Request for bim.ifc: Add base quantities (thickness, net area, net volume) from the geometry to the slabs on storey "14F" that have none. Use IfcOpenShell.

First a look at what the model holds.

```python
import ifcopenshell
import ifcopenshell.util.element
import ifcopenshell.util.unit

model = ifcopenshell.open("bim.ifc")
print(model.schema)
for unit_type in ("LENGTHUNIT", "AREAUNIT", "VOLUMEUNIT"):
    print(unit_type, ifcopenshell.util.unit.calculate_unit_scale(model, unit_type))
storey = next(s for s in model.by_type("IfcBuildingStorey") if s.Name == "14F")
slabs = [e for e in ifcopenshell.util.element.get_decomposition(storey) if e.is_a("IfcSlab")]
for e in sorted(slabs, key=lambda e: e.id()):
    print(e.id(), e.is_a(), e.Name, list(ifcopenshell.util.element.get_psets(e, qtos_only=True)), sep=" | ")
```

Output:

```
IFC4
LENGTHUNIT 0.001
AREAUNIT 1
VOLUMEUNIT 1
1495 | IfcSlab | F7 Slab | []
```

```python
import ifcopenshell
import ifcopenshell.api.pset
import ifcopenshell.geom
import ifcopenshell.util.element
import ifcopenshell.util.shape
import ifcopenshell.util.unit

model = ifcopenshell.open("bim.ifc")
unit_scale = ifcopenshell.util.unit.calculate_unit_scale(model)
area_scale = ifcopenshell.util.unit.calculate_unit_scale(model, "AREAUNIT")
volume_scale = ifcopenshell.util.unit.calculate_unit_scale(model, "VOLUMEUNIT")
settings = ifcopenshell.geom.settings()

storey = next(s for s in model.by_type("IfcBuildingStorey") if s.Name == "14F")
slabs = [e for e in ifcopenshell.util.element.get_decomposition(storey) if e.is_a("IfcSlab")]

for e in sorted(slabs, key=lambda e: e.id()):
    if ifcopenshell.util.element.get_psets(e, qtos_only=True, should_inherit=False):
        continue
    # Geometry comes back in metres, in the element's own axes.
    shape = ifcopenshell.geom.create_shape(settings, e)
    values = {
        "Width": ifcopenshell.util.shape.get_z(shape.geometry) / unit_scale,
        "NetArea": ifcopenshell.util.shape.get_footprint_area(shape.geometry) / area_scale,
        "NetVolume": ifcopenshell.util.shape.get_volume(shape.geometry) / volume_scale,
    }
    qto = ifcopenshell.api.pset.add_qto(model, product=e, name="Qto_SlabBaseQuantities")
    ifcopenshell.api.pset.edit_qto(model, qto=qto, properties=values)
    print(e.id(), {k: round(v, 3) for k, v in values.items()})

model.write("bim_v2.ifc")
```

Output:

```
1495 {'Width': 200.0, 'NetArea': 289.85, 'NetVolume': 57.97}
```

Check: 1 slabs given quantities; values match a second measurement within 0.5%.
